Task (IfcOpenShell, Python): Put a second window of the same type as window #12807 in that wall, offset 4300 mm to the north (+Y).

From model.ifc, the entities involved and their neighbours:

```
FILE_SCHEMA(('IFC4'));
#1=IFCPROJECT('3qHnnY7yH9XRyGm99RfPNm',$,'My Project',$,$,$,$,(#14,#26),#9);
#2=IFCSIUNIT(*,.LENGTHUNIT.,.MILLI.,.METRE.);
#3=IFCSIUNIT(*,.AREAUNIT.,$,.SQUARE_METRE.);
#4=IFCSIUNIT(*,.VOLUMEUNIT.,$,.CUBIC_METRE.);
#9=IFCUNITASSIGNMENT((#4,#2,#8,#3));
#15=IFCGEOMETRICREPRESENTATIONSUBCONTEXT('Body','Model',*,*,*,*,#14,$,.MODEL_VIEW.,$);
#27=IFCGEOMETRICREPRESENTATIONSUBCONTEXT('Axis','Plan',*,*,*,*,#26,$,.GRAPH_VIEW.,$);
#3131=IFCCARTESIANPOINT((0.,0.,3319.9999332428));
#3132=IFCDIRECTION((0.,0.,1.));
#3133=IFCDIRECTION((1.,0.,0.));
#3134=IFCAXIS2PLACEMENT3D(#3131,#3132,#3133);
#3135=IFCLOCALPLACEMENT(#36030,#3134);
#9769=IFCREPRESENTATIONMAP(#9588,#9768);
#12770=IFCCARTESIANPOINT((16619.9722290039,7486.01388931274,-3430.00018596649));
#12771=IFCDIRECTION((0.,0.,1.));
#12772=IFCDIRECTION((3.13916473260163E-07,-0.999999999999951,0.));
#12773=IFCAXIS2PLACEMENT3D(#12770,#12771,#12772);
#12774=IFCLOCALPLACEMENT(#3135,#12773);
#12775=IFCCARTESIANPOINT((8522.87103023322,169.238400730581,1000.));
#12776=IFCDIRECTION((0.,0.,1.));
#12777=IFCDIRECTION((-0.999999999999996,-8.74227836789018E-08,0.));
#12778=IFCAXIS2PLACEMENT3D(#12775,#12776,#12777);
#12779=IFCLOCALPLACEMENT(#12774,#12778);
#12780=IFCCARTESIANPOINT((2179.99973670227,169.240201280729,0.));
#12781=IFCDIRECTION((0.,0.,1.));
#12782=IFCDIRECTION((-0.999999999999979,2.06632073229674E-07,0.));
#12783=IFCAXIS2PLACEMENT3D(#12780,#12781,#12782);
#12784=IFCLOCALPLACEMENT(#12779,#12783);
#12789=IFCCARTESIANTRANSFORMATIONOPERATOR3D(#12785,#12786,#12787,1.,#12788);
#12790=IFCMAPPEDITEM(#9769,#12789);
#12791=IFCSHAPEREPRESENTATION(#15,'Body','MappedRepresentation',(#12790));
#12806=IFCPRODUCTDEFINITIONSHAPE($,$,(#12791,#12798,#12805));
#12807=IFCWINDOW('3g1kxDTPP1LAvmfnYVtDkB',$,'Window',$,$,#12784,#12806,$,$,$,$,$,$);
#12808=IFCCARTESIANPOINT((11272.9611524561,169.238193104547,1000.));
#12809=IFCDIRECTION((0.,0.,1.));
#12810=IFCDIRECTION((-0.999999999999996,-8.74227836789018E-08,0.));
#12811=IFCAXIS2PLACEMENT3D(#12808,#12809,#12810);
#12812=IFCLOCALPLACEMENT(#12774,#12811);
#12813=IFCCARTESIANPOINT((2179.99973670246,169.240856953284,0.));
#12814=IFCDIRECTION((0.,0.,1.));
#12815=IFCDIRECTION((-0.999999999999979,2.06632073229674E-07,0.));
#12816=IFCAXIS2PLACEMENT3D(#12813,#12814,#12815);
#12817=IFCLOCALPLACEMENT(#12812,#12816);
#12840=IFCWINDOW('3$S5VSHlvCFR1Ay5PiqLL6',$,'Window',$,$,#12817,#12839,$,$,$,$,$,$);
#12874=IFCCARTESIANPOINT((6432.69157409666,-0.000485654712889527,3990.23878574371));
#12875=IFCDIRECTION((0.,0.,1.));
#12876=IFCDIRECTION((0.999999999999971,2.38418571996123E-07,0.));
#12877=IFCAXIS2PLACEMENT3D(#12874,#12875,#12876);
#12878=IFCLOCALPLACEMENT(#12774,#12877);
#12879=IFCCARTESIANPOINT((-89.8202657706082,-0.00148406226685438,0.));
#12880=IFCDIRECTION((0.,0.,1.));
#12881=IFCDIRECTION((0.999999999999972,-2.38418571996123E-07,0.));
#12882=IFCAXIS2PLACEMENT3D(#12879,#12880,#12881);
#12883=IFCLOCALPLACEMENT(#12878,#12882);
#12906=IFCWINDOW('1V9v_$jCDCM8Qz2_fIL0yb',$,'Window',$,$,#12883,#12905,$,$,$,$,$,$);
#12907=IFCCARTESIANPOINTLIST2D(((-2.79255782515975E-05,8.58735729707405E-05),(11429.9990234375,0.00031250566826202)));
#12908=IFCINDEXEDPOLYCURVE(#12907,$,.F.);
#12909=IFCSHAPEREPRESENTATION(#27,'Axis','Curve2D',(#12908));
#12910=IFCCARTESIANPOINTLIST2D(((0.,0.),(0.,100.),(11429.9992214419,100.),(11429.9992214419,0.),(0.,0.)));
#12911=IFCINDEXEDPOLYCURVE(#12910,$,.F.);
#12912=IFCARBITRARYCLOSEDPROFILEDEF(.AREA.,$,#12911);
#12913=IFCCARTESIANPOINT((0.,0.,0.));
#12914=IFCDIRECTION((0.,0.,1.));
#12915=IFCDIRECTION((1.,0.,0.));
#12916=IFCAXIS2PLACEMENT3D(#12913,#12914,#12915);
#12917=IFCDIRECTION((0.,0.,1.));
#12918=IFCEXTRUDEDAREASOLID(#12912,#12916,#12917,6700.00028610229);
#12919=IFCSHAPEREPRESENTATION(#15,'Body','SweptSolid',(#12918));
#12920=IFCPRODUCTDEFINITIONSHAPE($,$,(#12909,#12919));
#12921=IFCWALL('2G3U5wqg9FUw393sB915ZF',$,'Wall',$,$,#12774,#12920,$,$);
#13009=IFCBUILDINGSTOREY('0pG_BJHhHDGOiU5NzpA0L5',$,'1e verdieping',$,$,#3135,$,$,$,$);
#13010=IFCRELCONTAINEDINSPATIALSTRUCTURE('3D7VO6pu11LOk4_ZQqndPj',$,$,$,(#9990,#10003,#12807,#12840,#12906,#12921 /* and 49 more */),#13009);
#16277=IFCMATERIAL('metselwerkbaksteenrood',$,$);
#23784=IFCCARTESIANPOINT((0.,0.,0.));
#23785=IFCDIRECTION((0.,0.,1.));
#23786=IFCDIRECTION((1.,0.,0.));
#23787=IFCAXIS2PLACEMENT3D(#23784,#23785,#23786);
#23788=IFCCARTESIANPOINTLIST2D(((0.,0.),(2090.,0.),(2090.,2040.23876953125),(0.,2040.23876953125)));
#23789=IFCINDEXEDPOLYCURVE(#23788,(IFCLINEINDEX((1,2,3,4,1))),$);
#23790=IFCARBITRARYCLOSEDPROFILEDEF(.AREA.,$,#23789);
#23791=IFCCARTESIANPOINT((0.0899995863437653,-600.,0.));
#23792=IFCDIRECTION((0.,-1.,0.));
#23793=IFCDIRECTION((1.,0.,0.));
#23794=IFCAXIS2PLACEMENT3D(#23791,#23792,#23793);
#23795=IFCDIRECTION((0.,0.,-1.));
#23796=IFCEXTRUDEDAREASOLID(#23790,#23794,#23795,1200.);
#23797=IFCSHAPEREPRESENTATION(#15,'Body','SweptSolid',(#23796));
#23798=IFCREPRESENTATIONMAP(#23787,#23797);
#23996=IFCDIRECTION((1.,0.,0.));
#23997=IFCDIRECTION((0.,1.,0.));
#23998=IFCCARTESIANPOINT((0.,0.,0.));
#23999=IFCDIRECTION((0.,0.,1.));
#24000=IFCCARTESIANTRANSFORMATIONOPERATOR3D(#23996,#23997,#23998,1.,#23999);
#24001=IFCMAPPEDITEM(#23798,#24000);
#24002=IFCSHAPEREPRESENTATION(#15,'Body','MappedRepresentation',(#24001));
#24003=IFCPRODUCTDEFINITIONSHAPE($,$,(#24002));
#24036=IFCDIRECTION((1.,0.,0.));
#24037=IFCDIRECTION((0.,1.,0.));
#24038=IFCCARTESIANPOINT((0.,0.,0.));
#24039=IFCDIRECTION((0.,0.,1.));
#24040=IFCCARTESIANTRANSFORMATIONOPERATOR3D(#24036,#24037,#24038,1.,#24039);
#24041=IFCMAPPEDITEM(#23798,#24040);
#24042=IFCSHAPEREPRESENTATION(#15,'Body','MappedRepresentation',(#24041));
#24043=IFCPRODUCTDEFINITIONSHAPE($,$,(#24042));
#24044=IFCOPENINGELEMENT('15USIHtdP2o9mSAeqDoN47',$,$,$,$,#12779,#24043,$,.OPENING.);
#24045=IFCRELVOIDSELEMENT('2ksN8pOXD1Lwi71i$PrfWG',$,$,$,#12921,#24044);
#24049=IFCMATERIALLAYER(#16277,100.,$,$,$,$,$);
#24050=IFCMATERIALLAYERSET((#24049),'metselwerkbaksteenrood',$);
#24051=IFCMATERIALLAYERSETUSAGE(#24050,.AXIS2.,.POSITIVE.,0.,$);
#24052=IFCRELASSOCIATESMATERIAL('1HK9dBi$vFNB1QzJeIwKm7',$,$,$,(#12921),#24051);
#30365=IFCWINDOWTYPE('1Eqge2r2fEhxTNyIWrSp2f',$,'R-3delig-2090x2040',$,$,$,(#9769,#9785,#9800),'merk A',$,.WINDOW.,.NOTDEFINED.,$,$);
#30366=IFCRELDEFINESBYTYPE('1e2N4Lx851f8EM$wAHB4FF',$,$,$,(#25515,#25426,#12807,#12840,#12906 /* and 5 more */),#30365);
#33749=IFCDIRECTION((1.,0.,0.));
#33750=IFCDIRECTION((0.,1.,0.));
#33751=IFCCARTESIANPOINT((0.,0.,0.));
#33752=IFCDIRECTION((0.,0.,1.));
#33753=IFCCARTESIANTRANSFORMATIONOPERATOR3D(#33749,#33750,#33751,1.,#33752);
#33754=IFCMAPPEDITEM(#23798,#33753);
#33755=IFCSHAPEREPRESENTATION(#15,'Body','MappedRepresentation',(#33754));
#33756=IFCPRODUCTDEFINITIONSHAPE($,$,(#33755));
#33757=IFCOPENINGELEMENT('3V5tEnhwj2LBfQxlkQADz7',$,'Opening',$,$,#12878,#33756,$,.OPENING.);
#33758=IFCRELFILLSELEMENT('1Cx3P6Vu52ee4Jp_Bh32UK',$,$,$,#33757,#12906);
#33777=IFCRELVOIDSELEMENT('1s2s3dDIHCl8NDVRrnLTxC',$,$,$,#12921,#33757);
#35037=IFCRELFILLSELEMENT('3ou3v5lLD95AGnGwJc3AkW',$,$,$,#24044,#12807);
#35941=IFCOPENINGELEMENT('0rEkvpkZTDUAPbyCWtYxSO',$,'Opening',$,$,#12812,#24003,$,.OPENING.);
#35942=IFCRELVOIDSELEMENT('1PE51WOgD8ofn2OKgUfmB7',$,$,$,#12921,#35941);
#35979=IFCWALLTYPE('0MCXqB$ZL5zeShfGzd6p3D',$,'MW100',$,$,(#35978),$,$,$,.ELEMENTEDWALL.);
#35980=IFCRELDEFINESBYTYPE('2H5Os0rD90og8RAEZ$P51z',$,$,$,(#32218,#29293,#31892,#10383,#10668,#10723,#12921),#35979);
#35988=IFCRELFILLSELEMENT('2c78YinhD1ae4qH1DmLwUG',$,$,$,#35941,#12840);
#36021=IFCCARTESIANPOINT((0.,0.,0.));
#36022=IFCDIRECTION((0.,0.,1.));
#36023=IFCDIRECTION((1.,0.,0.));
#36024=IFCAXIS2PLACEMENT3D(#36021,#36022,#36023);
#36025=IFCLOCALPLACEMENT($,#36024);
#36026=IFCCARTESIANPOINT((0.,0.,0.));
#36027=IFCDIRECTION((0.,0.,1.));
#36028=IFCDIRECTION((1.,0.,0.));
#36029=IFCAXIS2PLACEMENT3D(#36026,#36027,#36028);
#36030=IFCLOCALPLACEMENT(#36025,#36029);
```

```python
import ifcopenshell
import ifcopenshell.api.feature
import ifcopenshell.api.geometry
import ifcopenshell.api.root
import ifcopenshell.geom
import ifcopenshell.util.element
import ifcopenshell.util.placement
import ifcopenshell.util.shape
import ifcopenshell.util.unit

model = ifcopenshell.open("model.ifc")
unit_scale = ifcopenshell.util.unit.calculate_unit_scale(model)
settings = ifcopenshell.geom.settings()


def volume(element):
    """Net volume in cubic metres, openings subtracted."""
    shape = ifcopenshell.geom.create_shape(settings, element)
    return ifcopenshell.util.shape.get_volume(shape.geometry)


window = model.by_guid("3g1kxDTPP1LAvmfnYVtDkB")
opening = window.FillsVoids[0].RelatingOpeningElement
wall = opening.VoidsElements[0].RelatingBuildingElement
before = volume(wall)
shift = ifcopenshell.util.placement.get_local_placement(wall.ObjectPlacement)[:3, 0] * -4.3 / unit_scale

# copy_class copies the void relationship, type, container and properties, but no geometry.
new_opening = ifcopenshell.api.root.copy_class(model, product=opening)
new_opening.Representation = ifcopenshell.util.element.copy_deep(
    model, opening.Representation, exclude=["IfcGeometricRepresentationContext", "IfcRepresentationMap"]
)
new_window = ifcopenshell.api.root.copy_class(model, product=window)
new_window.Representation = ifcopenshell.util.element.copy_deep(
    model, window.Representation, exclude=["IfcGeometricRepresentationContext", "IfcRepresentationMap"]
)
ifcopenshell.api.feature.add_filling(model, opening=new_opening, element=new_window)

for old, new in ((opening, new_opening), (window, new_window)):
    matrix = ifcopenshell.util.placement.get_local_placement(old.ObjectPlacement)
    matrix[:3, 3] += shift
    ifcopenshell.api.geometry.edit_object_placement(model, product=new, matrix=matrix, is_si=False)

after = volume(wall)

print(f"wall volume {before:.3f} -> {after:.3f} m3")

model.write("model-out.ifc")
```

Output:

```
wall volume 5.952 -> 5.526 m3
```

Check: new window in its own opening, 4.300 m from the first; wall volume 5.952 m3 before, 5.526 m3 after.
